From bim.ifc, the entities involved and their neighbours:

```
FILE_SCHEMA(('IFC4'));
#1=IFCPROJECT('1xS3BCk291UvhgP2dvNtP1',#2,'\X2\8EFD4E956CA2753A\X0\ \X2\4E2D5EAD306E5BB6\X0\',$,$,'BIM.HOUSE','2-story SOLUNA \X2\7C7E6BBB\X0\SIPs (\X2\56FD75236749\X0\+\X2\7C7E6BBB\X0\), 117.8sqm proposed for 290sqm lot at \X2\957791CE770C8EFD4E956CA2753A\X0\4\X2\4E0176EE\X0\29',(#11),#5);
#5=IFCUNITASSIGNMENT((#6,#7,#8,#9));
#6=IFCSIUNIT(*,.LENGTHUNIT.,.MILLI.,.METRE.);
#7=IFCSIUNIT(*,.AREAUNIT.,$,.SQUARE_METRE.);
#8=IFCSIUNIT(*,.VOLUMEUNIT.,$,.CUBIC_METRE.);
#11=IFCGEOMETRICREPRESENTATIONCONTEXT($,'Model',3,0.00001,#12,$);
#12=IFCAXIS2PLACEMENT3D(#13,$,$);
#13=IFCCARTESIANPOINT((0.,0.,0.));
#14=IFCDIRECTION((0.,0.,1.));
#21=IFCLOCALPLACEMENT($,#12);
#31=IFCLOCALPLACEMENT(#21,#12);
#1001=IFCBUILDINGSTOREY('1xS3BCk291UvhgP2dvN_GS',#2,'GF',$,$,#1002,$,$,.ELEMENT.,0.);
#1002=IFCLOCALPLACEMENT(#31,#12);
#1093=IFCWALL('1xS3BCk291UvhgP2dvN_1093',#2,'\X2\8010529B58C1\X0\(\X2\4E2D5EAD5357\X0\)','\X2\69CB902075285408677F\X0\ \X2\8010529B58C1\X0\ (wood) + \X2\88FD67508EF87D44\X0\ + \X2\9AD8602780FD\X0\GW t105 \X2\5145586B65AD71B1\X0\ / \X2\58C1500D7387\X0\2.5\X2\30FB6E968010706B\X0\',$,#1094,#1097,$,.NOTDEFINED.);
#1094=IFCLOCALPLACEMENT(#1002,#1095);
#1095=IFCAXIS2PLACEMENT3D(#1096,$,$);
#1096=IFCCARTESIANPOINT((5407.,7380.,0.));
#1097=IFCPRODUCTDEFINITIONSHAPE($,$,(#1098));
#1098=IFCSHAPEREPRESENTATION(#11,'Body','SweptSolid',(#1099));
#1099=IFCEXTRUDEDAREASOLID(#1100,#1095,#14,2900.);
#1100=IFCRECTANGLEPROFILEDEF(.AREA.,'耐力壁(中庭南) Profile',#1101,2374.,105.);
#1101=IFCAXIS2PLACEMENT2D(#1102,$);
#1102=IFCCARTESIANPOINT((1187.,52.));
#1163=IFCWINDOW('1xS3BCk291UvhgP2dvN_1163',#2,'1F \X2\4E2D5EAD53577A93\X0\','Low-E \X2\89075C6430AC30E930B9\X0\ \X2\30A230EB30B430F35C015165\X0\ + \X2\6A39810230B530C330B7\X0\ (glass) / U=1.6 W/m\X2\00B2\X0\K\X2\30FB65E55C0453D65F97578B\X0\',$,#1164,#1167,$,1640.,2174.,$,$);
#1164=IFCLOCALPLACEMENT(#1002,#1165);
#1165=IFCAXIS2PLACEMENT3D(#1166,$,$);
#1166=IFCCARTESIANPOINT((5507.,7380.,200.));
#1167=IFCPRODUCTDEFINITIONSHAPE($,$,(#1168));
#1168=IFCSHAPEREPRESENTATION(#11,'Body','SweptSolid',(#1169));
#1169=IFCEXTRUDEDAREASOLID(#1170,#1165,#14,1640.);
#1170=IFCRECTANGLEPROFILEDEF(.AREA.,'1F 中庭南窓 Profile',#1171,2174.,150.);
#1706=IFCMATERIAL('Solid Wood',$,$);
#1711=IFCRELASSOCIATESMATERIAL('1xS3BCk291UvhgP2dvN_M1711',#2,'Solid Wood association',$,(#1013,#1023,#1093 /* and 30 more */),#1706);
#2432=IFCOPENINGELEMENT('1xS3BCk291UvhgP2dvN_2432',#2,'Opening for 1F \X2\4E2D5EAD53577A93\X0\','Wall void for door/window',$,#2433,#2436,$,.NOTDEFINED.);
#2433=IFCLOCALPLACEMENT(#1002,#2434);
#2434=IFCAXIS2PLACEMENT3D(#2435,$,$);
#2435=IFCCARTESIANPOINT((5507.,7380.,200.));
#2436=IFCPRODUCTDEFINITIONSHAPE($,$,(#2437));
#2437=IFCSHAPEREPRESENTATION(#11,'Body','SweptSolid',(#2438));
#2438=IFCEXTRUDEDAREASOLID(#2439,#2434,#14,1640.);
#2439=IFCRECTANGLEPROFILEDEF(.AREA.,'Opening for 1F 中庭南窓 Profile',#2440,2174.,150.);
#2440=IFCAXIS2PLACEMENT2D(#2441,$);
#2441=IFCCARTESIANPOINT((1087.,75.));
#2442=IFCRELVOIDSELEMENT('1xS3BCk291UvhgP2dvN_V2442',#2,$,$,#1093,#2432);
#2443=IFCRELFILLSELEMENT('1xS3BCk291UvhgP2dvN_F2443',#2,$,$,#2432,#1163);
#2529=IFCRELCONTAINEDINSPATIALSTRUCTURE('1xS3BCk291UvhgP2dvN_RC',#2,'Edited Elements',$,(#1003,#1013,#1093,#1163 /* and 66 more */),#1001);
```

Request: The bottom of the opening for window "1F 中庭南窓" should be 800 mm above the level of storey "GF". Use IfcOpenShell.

```python
import numpy as np
import ifcopenshell
import ifcopenshell.api.geometry
import ifcopenshell.geom
import ifcopenshell.util.element
import ifcopenshell.util.placement
import ifcopenshell.util.shape
import ifcopenshell.util.unit

model = ifcopenshell.open("bim.ifc")
unit_scale = ifcopenshell.util.unit.calculate_unit_scale(model)

window = model.by_guid("1xS3BCk291UvhgP2dvN_1163")
opening = window.FillsVoids[0].RelatingOpeningElement
storey = ifcopenshell.util.element.get_container(window, ifc_class="IfcBuildingStorey")
level = ifcopenshell.util.placement.get_local_placement(storey.ObjectPlacement)[2, 3]

# The opening's origin need not be at the sill, so measure its lowest point.
shape = ifcopenshell.geom.create_shape(ifcopenshell.geom.settings(), opening)
bottom = ifcopenshell.util.shape.get_shape_bottom_elevation(shape, shape.geometry) / unit_scale
dz = level + 800.0 - bottom

shift = np.array([0.0, 0.0, dz])
# The window is not placed relative to its opening, so move both.
for product in (opening, window):
    matrix = ifcopenshell.util.placement.get_local_placement(product.ObjectPlacement)
    matrix[:3, 3] += shift
    ifcopenshell.api.geometry.edit_object_placement(model, product=product, matrix=matrix, is_si=False)

print(f"moved by {dz * unit_scale:+.3f} m")

model.write("bim_v2.ifc")
```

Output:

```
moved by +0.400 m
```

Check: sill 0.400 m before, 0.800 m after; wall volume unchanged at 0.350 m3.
